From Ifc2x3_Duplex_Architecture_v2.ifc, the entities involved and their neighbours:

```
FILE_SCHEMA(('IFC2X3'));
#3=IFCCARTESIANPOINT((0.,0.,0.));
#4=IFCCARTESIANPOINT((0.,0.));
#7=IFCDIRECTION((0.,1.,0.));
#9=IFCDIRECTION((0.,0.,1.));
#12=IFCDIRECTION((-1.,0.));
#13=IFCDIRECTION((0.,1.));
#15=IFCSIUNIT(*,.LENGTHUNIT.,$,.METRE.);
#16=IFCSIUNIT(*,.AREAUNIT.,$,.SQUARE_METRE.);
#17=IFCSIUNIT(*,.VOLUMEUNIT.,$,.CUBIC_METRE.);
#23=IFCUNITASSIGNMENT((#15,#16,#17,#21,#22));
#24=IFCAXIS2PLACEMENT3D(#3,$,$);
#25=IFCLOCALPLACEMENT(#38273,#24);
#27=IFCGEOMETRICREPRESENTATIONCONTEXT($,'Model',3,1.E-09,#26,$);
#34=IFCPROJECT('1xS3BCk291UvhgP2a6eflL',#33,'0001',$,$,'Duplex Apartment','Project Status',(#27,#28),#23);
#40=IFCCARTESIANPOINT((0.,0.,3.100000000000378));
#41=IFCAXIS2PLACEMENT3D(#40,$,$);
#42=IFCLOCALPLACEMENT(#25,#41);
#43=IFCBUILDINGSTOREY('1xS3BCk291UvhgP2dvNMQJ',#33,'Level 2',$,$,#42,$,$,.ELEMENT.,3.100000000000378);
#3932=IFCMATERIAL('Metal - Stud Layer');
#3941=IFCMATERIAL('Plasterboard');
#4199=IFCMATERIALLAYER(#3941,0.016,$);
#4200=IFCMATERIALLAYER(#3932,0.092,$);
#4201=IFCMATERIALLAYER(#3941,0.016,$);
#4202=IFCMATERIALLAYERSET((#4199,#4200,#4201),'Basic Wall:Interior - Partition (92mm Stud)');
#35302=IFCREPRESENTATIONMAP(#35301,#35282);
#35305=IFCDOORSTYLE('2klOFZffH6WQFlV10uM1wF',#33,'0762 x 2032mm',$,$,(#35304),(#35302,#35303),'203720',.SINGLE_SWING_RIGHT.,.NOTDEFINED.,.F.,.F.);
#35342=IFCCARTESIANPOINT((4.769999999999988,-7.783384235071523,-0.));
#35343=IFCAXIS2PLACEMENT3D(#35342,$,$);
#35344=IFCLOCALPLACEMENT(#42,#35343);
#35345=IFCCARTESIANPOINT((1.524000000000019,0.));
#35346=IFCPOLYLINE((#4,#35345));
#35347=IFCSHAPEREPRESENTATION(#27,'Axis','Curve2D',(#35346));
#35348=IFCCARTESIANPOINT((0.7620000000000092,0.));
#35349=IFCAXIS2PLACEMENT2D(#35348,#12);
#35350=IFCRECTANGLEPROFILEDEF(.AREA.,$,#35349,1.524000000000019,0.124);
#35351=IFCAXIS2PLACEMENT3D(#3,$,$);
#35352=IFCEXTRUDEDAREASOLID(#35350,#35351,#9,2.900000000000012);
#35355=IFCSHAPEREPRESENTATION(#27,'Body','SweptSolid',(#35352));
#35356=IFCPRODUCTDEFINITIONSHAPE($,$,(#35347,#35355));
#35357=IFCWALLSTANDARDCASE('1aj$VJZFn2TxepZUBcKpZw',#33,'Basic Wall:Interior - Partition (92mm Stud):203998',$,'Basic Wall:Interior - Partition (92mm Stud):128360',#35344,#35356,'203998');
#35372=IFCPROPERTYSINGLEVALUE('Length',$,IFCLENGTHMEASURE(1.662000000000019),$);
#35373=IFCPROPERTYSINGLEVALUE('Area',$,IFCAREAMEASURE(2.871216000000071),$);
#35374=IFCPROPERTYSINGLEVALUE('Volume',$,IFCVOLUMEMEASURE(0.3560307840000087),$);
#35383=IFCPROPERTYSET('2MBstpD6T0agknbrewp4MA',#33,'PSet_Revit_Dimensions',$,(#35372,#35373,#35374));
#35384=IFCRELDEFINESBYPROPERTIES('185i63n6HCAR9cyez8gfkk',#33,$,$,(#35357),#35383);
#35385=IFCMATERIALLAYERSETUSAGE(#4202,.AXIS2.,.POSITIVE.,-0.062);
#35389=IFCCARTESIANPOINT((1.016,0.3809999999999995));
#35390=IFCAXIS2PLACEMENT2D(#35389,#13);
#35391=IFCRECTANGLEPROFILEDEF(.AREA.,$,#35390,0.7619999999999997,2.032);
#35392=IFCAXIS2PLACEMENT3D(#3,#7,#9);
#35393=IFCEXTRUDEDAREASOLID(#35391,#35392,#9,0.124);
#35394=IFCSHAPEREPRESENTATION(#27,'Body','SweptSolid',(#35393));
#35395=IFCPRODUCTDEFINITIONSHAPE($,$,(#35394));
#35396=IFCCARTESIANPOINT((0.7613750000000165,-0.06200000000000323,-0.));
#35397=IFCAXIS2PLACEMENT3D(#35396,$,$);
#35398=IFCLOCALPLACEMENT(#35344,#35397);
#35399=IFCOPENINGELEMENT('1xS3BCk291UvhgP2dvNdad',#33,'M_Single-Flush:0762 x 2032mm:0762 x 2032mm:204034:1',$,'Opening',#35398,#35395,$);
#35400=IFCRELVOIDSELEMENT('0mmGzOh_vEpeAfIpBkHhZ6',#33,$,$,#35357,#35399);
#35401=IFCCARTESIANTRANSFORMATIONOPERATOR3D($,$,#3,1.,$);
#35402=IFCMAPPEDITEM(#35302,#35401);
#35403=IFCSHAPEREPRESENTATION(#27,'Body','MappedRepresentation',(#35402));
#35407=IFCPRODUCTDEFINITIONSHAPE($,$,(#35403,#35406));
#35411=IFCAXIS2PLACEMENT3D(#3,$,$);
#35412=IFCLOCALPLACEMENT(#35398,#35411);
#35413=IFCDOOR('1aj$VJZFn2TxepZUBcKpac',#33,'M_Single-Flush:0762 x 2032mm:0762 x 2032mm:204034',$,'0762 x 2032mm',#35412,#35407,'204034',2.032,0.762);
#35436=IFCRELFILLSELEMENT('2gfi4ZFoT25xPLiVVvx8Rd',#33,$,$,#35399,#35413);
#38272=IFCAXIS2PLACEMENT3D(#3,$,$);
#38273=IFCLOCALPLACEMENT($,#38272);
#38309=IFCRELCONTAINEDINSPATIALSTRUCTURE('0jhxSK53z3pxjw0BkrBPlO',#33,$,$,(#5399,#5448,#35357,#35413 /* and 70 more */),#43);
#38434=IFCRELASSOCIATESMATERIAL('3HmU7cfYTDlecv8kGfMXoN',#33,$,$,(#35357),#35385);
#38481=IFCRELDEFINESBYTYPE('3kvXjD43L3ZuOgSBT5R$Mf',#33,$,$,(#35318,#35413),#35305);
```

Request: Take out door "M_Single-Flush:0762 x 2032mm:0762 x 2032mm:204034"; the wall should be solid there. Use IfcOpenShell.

```python
import ifcopenshell
import ifcopenshell.api.feature
import ifcopenshell.api.pset
import ifcopenshell.api.root
import ifcopenshell.geom
import ifcopenshell.util.element
import ifcopenshell.util.shape
import ifcopenshell.util.unit

model = ifcopenshell.open("Ifc2x3_Duplex_Architecture_v2.ifc")
area_scale = ifcopenshell.util.unit.calculate_unit_scale(model, "AREAUNIT")
volume_scale = ifcopenshell.util.unit.calculate_unit_scale(model, "VOLUMEUNIT")
settings = ifcopenshell.geom.settings()


def volume(element):
    """Net volume in cubic metres, openings subtracted."""
    shape = ifcopenshell.geom.create_shape(settings, element)
    return ifcopenshell.util.shape.get_volume(shape.geometry)


door = model.by_guid("1aj$VJZFn2TxepZUBcKpac")
opening = door.FillsVoids[0].RelatingOpeningElement
wall = opening.VoidsElements[0].RelatingBuildingElement
before = volume(wall)

ifcopenshell.api.root.remove_product(model, product=door)
ifcopenshell.api.feature.remove_feature(model, feature=opening)

after = volume(wall)
thickness = 0.124  # wall thickness in metres

# Update the wall's stored quantities.
pset = model.by_id(ifcopenshell.util.element.get_pset(wall, "PSet_Revit_Dimensions", should_inherit=False)["id"])
ifcopenshell.api.pset.edit_pset(model, pset=pset, properties={
    "Area": model.create_entity("IfcAreaMeasure", after / thickness / area_scale),
    "Volume": model.create_entity("IfcVolumeMeasure", after / volume_scale),
})

print(f"wall volume {before:.3f} -> {after:.3f} m3")

model.write("Ifc2x3_Duplex_Architecture_v2-out.ifc")
```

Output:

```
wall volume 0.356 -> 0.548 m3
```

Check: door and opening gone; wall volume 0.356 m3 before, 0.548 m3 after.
